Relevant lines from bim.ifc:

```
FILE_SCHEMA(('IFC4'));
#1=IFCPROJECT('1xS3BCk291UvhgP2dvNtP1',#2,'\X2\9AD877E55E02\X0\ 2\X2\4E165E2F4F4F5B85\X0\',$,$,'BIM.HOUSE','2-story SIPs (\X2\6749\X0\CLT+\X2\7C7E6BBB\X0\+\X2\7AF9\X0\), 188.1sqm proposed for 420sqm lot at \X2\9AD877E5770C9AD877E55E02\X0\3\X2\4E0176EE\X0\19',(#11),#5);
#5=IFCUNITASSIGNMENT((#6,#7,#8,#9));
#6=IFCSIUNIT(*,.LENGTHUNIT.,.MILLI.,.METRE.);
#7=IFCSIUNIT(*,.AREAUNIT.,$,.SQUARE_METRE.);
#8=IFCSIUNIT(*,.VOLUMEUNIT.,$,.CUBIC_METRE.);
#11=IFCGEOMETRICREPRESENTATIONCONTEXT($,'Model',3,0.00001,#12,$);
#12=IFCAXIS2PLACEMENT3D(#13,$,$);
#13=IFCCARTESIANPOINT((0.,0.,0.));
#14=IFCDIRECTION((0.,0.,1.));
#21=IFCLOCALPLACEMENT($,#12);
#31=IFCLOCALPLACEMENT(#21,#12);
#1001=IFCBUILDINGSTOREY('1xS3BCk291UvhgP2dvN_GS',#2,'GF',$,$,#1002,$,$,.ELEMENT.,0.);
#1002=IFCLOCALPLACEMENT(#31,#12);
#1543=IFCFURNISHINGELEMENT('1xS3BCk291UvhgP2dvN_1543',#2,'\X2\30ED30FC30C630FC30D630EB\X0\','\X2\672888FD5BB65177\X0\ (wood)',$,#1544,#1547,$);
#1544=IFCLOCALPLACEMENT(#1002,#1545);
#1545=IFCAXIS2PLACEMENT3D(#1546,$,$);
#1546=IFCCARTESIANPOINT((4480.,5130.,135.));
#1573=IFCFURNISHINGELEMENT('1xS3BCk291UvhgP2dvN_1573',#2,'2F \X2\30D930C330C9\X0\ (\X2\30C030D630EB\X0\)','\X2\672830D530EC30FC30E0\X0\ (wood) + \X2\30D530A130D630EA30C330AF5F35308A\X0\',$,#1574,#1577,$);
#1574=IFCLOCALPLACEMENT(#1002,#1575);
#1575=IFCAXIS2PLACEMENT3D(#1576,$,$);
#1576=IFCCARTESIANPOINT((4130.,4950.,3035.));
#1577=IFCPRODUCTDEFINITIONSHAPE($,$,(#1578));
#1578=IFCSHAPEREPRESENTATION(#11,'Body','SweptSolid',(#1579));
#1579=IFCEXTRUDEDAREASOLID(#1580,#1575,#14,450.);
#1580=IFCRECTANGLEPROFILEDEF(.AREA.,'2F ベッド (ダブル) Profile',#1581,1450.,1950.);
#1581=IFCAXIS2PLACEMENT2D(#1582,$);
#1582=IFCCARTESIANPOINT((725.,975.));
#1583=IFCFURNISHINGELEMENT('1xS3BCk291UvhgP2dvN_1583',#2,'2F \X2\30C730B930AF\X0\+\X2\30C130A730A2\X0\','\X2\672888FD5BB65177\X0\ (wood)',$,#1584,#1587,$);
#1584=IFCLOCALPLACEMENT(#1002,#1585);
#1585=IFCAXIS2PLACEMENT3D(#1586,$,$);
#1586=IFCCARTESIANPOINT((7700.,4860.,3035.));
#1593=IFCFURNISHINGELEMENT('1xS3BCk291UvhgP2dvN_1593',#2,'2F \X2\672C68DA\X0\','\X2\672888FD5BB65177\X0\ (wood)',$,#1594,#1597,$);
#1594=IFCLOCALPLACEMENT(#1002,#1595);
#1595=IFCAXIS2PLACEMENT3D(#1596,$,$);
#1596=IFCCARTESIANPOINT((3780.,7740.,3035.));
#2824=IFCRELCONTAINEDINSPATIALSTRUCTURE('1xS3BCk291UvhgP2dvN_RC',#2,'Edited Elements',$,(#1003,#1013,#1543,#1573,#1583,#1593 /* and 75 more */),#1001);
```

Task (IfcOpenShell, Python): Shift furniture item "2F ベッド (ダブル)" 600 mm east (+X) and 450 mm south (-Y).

```python
import ifcopenshell
import ifcopenshell.api.geometry
import ifcopenshell.util.placement
import ifcopenshell.util.unit

model = ifcopenshell.open("bim.ifc")
unit_scale = ifcopenshell.util.unit.calculate_unit_scale(model)

item = model.by_guid("1xS3BCk291UvhgP2dvN_1573")
matrix = ifcopenshell.util.placement.get_local_placement(item.ObjectPlacement)
matrix[0, 3] += 0.6 / unit_scale
matrix[1, 3] -= 0.45 / unit_scale
ifcopenshell.api.geometry.edit_object_placement(model, product=item, matrix=matrix, is_si=False)

print(ifcopenshell.util.placement.get_local_placement(item.ObjectPlacement).round(3) + 0.0)

model.write("bim_edited.ifc")
```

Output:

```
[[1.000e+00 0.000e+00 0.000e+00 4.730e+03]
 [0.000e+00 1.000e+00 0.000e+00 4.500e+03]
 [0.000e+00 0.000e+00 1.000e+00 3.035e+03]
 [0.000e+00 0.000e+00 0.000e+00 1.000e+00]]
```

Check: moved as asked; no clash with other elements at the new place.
